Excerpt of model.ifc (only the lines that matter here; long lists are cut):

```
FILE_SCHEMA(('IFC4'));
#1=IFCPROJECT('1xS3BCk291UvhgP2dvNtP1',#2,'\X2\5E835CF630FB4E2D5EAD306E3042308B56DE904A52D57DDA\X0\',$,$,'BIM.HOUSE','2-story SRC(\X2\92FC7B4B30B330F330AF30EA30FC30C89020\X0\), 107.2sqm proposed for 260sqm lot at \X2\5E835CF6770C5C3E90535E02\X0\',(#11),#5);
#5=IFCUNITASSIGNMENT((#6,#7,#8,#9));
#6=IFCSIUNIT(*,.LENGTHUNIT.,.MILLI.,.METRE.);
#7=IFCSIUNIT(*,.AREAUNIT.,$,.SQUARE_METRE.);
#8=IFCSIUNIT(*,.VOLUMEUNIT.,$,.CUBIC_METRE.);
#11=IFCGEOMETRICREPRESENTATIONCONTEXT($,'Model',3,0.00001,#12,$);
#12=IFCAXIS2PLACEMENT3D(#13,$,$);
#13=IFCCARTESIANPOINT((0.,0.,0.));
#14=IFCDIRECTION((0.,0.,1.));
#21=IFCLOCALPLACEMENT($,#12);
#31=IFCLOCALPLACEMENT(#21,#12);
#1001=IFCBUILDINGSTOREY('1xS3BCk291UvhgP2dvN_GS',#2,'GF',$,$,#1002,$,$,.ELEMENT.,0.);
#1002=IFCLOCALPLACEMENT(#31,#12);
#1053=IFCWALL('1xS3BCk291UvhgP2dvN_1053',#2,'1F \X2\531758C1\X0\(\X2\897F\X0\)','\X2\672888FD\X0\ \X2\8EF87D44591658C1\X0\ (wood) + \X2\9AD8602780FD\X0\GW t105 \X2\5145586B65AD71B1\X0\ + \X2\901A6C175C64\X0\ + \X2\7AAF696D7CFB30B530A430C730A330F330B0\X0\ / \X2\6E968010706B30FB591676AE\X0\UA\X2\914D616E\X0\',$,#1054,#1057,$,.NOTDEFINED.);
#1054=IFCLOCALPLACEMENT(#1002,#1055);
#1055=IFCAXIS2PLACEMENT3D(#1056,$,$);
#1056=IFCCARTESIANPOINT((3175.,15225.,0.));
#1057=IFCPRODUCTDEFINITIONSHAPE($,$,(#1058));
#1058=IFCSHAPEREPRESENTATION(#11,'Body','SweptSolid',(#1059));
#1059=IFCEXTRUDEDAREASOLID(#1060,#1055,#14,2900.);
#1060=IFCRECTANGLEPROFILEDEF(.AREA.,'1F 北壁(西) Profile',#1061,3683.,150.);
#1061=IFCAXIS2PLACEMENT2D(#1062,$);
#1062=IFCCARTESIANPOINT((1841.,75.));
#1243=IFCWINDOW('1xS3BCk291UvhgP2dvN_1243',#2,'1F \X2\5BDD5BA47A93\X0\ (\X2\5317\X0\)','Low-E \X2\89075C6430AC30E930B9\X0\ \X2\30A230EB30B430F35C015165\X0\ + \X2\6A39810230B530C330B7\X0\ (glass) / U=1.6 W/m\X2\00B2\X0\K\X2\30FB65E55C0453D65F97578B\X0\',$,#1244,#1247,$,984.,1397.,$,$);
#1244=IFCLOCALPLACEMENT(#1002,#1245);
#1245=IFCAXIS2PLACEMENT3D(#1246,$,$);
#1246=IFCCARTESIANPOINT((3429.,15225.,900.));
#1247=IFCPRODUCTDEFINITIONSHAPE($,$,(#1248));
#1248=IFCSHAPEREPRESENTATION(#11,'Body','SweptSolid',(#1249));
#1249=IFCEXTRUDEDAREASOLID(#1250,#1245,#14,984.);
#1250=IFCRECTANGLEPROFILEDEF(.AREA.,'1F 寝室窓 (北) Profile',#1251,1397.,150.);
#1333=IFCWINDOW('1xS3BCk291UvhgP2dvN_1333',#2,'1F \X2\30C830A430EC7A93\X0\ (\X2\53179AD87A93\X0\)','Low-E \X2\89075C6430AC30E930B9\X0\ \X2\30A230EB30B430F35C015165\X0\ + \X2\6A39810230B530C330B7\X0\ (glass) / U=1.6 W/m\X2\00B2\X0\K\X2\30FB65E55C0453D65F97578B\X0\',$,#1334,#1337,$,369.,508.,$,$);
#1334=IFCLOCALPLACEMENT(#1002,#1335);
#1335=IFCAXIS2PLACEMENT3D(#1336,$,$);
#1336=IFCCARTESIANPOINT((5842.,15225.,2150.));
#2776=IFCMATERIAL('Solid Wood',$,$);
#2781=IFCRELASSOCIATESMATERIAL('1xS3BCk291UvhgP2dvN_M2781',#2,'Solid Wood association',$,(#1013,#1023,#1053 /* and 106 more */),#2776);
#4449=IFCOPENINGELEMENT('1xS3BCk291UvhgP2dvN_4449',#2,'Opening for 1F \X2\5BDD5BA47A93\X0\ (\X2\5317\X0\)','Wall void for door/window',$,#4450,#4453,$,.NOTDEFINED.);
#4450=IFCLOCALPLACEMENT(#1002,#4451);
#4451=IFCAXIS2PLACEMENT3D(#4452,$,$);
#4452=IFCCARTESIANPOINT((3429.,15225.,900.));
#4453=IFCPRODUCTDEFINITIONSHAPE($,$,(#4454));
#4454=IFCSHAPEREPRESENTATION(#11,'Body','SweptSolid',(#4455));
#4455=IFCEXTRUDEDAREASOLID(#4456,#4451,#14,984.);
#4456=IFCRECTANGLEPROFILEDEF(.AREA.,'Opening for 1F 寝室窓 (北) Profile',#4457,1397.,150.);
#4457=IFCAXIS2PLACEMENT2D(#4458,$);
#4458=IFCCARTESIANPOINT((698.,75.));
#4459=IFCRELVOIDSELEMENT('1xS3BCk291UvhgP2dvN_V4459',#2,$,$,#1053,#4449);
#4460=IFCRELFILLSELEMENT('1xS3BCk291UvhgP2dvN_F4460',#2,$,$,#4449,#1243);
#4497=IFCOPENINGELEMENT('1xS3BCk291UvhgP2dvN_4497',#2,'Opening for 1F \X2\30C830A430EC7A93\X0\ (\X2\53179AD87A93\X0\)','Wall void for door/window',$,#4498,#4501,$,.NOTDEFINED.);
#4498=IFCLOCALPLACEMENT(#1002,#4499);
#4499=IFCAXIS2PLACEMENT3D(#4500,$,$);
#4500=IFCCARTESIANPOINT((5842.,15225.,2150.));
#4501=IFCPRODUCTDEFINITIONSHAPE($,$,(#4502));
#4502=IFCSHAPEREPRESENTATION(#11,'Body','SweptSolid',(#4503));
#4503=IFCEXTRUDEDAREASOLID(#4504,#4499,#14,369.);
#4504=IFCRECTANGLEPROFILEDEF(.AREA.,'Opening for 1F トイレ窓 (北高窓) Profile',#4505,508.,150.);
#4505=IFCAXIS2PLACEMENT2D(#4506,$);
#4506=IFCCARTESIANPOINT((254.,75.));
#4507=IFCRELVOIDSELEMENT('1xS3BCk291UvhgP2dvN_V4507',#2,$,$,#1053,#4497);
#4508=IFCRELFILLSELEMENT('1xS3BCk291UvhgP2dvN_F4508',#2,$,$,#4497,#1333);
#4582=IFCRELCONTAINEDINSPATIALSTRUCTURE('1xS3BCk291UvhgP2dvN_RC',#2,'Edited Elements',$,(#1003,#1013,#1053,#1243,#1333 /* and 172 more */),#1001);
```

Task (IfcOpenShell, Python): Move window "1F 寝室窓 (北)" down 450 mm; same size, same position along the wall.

```python
import numpy as np
import ifcopenshell
import ifcopenshell.api.geometry
import ifcopenshell.util.placement
import ifcopenshell.util.unit

model = ifcopenshell.open("model.ifc")
unit_scale = ifcopenshell.util.unit.calculate_unit_scale(model)

window = model.by_guid("1xS3BCk291UvhgP2dvN_1243")
opening = window.FillsVoids[0].RelatingOpeningElement
dz = -0.45 / unit_scale

shift = np.array([0.0, 0.0, dz])
# The window is not placed relative to its opening, so move both.
for product in (opening, window):
    matrix = ifcopenshell.util.placement.get_local_placement(product.ObjectPlacement)
    matrix[:3, 3] += shift
    ifcopenshell.api.geometry.edit_object_placement(model, product=product, matrix=matrix, is_si=False)

print(f"moved by {dz * unit_scale:+.3f} m")

model.write("model_edited.ifc")
```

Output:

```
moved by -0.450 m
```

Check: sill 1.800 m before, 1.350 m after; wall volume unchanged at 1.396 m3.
